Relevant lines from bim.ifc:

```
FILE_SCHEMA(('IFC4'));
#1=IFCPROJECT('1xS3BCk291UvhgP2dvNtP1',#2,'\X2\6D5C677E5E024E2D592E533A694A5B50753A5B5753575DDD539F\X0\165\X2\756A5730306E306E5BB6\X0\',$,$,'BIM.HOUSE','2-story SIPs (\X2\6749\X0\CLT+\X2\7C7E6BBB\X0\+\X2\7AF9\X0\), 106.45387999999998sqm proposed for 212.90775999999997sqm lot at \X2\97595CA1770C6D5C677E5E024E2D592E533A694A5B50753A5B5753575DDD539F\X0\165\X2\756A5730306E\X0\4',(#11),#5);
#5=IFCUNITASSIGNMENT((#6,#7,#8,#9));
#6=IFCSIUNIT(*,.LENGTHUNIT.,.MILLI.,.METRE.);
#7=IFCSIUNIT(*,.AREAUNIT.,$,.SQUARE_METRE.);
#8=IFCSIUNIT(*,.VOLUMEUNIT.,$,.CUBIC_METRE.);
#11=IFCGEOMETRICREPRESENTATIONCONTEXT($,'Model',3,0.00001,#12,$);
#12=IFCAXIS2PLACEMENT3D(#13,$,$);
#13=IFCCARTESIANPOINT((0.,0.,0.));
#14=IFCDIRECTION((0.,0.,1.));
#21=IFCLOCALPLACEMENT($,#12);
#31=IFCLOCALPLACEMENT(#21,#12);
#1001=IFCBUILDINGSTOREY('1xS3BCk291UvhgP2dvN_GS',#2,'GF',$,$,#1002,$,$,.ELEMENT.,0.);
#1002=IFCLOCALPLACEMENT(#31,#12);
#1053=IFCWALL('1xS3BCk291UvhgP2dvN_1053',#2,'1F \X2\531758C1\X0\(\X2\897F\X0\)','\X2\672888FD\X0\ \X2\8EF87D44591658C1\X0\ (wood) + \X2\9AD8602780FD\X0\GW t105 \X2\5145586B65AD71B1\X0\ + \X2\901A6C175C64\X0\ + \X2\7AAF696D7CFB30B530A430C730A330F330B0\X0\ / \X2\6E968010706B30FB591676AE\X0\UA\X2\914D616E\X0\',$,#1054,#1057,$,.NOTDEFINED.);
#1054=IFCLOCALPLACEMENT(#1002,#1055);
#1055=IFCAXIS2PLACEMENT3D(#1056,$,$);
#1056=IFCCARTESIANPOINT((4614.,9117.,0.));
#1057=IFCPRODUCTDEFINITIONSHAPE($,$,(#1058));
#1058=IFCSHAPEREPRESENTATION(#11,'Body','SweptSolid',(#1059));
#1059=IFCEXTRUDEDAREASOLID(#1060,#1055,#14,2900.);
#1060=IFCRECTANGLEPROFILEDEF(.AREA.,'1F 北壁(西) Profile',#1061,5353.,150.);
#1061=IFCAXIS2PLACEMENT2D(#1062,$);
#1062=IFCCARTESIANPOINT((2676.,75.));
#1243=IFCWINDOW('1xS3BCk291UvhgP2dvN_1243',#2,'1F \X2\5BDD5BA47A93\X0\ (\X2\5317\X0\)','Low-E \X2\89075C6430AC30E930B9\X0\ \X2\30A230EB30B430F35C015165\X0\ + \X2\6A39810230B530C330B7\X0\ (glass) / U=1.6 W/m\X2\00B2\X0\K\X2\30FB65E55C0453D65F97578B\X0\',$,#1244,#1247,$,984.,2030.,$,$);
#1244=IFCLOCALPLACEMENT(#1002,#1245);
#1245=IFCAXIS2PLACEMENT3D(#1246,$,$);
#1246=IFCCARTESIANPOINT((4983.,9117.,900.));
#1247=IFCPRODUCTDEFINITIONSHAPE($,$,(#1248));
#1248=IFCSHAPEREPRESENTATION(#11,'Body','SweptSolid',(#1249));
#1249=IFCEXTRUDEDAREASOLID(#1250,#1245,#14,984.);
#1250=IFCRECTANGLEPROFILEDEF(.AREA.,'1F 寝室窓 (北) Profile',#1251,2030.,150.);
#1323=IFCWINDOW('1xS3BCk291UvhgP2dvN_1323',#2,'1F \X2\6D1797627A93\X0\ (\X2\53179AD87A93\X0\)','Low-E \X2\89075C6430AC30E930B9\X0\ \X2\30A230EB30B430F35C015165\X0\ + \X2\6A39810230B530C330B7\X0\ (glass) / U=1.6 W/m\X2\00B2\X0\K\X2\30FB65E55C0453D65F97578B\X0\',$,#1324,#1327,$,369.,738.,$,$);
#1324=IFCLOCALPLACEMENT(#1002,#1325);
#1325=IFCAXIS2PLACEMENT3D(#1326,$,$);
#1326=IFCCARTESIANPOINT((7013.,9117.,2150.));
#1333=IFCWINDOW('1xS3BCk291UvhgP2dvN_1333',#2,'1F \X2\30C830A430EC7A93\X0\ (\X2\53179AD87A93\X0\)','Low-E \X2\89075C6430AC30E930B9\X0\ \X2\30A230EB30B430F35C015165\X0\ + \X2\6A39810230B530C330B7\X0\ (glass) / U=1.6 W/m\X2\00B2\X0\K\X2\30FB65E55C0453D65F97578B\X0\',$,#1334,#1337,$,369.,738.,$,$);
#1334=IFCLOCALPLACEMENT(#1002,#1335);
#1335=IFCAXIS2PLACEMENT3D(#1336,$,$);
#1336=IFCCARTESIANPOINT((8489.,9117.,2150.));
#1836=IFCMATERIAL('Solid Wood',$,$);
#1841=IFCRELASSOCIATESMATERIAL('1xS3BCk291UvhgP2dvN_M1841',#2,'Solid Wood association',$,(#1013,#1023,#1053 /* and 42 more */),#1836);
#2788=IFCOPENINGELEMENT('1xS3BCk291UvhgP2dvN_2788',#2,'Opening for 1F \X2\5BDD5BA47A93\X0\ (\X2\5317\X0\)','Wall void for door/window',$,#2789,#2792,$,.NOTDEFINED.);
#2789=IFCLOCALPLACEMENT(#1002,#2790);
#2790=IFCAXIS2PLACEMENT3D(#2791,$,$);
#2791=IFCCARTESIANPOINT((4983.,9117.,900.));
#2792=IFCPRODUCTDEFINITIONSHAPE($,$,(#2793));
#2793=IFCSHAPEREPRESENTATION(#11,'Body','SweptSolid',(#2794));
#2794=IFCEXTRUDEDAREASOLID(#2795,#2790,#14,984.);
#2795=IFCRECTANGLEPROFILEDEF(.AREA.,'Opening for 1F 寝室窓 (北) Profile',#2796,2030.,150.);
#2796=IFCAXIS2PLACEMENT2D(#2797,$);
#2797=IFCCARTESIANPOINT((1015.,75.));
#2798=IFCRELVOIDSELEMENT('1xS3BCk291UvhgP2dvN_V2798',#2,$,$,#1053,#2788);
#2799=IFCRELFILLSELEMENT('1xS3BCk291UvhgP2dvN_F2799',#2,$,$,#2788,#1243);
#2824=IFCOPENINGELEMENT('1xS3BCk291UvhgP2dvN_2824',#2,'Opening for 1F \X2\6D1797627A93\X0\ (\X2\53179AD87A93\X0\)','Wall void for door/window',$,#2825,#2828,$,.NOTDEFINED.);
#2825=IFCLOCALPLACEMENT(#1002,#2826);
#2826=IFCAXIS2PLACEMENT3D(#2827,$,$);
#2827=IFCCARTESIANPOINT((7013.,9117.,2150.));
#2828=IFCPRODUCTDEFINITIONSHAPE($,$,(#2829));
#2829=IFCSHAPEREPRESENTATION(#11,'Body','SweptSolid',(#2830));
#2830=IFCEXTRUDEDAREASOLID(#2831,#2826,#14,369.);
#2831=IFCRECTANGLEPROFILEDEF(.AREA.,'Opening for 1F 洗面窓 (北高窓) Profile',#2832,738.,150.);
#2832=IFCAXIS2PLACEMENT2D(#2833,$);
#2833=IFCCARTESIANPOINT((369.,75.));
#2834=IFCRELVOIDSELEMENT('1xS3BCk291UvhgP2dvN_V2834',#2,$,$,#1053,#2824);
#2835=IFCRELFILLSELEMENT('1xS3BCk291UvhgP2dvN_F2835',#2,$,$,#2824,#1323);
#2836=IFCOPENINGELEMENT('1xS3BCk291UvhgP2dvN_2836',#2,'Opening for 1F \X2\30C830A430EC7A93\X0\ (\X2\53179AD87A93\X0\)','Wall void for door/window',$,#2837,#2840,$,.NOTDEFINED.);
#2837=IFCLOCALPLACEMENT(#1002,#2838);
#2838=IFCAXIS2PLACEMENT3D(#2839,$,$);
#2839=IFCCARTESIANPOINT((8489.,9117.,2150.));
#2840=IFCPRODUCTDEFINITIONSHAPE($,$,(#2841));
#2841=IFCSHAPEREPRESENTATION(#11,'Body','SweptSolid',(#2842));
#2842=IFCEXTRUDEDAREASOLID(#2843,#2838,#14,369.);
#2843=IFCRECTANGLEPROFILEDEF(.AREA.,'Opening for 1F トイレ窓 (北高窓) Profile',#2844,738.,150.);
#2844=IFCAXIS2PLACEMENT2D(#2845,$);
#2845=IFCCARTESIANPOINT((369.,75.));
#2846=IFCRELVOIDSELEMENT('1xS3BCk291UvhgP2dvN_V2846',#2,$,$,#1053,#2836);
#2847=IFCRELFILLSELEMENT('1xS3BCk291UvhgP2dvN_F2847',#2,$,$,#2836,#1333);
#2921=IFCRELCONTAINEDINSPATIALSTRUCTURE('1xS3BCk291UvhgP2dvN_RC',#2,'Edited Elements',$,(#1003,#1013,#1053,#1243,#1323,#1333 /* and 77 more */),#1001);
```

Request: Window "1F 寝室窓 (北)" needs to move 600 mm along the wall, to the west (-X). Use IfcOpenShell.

```python
import ifcopenshell
import ifcopenshell.api.geometry
import ifcopenshell.util.placement

model = ifcopenshell.open("bim.ifc")

window = model.by_id(1243)
opening = window.FillsVoids[0].RelatingOpeningElement
wall = opening.VoidsElements[0].RelatingBuildingElement

wall_matrix = ifcopenshell.util.placement.get_local_placement(wall.ObjectPlacement)
shift = wall_matrix[:3, 0] * -600.0
before = ifcopenshell.util.placement.get_local_placement(window.ObjectPlacement)[:3, 3].copy()

# The window is not placed relative to its opening, so move both.
for product in (opening, window):
    matrix = ifcopenshell.util.placement.get_local_placement(product.ObjectPlacement)
    matrix[:3, 3] += shift
    ifcopenshell.api.geometry.edit_object_placement(model, product=product, matrix=matrix, is_si=False)

after = ifcopenshell.util.placement.get_local_placement(window.ObjectPlacement)[:3, 3]
print("window moved by", (after - before).round(3) + 0.0)

model.write("bim_edited.ifc")
```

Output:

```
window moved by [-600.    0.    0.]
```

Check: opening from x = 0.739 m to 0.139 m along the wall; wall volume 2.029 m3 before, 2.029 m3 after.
